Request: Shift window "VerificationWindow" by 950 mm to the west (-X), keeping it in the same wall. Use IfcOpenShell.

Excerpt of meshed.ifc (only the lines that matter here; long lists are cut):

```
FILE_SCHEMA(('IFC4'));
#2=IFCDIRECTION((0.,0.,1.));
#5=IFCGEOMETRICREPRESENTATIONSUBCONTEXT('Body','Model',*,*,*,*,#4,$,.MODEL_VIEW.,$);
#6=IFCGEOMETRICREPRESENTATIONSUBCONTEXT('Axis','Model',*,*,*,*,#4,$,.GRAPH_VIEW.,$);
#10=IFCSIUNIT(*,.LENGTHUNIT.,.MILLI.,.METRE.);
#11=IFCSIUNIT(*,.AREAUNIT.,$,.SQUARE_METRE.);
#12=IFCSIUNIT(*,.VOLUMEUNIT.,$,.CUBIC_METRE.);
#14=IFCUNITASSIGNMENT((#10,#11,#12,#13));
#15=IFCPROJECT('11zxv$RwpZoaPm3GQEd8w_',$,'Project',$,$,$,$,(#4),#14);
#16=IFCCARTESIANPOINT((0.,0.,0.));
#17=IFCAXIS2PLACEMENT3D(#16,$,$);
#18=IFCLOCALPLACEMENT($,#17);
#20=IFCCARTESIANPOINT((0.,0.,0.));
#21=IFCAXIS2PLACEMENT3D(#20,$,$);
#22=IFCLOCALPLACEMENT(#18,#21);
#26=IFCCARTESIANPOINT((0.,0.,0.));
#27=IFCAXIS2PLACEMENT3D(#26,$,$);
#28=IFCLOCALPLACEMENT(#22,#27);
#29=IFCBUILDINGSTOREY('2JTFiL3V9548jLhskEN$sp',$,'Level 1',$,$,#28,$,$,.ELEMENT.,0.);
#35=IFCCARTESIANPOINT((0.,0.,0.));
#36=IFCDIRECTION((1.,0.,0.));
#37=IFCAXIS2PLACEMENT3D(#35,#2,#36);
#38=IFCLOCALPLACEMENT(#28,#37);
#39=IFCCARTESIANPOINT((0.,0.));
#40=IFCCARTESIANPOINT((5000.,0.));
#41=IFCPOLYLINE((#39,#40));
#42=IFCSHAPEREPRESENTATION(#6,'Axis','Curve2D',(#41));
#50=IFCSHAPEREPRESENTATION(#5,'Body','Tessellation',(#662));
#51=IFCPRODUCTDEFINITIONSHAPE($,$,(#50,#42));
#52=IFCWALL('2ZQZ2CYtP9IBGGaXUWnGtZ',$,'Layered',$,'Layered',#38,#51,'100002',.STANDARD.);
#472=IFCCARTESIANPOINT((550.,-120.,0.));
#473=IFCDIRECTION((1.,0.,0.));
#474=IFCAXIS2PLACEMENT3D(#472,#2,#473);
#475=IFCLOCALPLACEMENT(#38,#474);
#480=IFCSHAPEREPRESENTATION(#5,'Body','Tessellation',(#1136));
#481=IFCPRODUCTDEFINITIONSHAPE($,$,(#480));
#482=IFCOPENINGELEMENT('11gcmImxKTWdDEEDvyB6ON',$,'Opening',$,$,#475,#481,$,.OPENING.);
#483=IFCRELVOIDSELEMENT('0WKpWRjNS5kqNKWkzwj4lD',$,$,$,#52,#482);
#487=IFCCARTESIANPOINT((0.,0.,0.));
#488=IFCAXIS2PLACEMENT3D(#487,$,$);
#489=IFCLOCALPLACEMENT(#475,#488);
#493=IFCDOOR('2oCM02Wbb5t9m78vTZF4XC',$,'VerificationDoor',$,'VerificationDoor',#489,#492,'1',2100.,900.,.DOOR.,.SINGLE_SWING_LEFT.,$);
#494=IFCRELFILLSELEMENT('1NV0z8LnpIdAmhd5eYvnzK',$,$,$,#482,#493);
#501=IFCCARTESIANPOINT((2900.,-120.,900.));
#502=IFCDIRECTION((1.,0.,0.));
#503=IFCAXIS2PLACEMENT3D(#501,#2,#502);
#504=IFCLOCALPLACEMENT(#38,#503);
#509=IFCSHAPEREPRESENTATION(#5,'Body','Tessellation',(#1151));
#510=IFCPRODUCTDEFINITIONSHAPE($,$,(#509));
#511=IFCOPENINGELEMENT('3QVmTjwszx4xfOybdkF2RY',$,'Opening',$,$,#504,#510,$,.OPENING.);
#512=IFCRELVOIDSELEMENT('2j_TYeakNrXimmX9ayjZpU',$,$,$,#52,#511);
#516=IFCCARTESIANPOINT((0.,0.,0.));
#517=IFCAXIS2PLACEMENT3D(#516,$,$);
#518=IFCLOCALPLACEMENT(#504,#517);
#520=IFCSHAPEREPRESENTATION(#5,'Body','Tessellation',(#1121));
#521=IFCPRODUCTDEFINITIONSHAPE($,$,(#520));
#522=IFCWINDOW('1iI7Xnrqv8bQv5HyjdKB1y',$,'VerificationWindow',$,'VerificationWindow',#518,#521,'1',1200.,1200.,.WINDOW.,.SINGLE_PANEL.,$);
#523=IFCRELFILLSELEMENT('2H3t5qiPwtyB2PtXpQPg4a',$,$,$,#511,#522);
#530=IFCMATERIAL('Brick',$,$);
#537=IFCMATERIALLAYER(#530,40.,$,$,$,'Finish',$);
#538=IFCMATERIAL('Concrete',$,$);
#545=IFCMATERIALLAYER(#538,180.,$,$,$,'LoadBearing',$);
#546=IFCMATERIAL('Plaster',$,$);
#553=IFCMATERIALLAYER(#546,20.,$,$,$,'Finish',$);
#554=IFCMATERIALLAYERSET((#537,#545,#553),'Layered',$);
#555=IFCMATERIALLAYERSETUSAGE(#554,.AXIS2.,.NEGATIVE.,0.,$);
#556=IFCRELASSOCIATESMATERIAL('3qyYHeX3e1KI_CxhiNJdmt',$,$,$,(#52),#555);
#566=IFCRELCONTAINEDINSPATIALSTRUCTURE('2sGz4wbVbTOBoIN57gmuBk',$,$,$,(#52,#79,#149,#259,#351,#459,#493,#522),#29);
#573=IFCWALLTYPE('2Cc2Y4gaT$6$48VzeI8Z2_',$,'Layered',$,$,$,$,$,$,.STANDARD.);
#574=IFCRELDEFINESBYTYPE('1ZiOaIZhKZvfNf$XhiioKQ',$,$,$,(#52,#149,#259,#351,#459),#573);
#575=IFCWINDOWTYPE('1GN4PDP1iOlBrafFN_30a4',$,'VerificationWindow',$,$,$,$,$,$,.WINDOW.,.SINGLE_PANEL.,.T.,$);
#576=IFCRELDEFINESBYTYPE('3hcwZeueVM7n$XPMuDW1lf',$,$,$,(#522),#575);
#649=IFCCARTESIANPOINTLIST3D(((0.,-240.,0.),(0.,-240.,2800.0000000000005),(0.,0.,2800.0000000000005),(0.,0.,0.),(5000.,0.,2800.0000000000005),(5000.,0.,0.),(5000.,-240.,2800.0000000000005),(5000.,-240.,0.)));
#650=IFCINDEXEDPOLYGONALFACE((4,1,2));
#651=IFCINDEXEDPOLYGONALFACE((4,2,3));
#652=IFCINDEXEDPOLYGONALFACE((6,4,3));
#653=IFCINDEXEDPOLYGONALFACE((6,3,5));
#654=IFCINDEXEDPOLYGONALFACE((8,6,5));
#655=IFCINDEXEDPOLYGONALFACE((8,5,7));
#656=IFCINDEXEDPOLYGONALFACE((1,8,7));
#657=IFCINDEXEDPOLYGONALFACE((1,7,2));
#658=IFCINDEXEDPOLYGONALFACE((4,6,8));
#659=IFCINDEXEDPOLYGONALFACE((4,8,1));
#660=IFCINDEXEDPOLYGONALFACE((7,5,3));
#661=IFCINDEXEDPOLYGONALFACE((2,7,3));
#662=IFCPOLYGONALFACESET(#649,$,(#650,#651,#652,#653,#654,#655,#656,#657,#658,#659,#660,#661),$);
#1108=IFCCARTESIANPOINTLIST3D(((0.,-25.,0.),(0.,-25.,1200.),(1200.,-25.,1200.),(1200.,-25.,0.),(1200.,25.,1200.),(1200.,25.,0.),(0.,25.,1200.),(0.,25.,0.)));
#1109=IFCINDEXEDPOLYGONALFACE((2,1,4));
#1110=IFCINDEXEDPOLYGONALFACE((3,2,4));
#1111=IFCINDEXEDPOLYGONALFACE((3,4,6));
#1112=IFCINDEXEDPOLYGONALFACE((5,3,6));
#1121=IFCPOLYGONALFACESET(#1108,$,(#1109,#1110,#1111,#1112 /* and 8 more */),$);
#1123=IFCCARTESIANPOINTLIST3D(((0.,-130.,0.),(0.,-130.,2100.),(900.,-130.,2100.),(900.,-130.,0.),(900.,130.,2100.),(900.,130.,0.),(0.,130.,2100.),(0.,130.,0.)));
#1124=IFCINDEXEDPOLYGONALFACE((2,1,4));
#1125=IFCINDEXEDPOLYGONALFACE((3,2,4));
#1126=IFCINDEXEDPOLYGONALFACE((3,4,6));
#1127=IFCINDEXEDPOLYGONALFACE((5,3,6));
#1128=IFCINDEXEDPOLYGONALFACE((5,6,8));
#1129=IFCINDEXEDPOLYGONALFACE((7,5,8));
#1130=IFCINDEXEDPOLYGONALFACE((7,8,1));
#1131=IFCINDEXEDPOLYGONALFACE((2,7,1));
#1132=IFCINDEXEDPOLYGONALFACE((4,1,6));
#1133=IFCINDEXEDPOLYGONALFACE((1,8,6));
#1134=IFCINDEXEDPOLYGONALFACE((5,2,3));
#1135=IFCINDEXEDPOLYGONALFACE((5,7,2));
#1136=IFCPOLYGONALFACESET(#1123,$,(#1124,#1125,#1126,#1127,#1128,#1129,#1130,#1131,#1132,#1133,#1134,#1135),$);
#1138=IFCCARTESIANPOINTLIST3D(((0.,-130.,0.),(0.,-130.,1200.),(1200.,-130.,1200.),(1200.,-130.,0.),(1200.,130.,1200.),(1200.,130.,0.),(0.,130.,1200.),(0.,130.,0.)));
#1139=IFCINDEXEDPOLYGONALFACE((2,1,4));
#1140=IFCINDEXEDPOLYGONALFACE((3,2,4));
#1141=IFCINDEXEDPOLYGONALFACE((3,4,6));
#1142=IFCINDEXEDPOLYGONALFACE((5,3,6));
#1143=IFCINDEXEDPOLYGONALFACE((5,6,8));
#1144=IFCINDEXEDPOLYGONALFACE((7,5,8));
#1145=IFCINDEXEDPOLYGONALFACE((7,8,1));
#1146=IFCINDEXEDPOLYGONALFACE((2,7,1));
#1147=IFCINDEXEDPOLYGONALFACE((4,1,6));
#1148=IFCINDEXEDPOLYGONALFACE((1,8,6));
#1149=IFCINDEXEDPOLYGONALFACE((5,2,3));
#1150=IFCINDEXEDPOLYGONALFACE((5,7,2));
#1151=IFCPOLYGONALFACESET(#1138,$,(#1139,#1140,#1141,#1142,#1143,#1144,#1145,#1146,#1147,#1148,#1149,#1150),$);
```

```python
import ifcopenshell
import ifcopenshell.api.geometry
import ifcopenshell.util.placement
import ifcopenshell.util.unit

model = ifcopenshell.open("meshed.ifc")
unit_scale = ifcopenshell.util.unit.calculate_unit_scale(model)

window = model.by_guid("1iI7Xnrqv8bQv5HyjdKB1y")
opening = window.FillsVoids[0].RelatingOpeningElement
wall = opening.VoidsElements[0].RelatingBuildingElement

wall_matrix = ifcopenshell.util.placement.get_local_placement(wall.ObjectPlacement)
shift = wall_matrix[:3, 0] * -0.95 / unit_scale
before = ifcopenshell.util.placement.get_local_placement(window.ObjectPlacement)[:3, 3].copy()

# The window is placed relative to its opening, so it follows when the opening moves.
matrix = ifcopenshell.util.placement.get_local_placement(opening.ObjectPlacement)
matrix[:3, 3] += shift
ifcopenshell.api.geometry.edit_object_placement(
    model, product=opening, matrix=matrix, is_si=False, should_transform_children=True
)

after = ifcopenshell.util.placement.get_local_placement(window.ObjectPlacement)[:3, 3]
print("window moved by", (after - before).round(3) + 0.0)

model.write("meshed-out.ifc")
```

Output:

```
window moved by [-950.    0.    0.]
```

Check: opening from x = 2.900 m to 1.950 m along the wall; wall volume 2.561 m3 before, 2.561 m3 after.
